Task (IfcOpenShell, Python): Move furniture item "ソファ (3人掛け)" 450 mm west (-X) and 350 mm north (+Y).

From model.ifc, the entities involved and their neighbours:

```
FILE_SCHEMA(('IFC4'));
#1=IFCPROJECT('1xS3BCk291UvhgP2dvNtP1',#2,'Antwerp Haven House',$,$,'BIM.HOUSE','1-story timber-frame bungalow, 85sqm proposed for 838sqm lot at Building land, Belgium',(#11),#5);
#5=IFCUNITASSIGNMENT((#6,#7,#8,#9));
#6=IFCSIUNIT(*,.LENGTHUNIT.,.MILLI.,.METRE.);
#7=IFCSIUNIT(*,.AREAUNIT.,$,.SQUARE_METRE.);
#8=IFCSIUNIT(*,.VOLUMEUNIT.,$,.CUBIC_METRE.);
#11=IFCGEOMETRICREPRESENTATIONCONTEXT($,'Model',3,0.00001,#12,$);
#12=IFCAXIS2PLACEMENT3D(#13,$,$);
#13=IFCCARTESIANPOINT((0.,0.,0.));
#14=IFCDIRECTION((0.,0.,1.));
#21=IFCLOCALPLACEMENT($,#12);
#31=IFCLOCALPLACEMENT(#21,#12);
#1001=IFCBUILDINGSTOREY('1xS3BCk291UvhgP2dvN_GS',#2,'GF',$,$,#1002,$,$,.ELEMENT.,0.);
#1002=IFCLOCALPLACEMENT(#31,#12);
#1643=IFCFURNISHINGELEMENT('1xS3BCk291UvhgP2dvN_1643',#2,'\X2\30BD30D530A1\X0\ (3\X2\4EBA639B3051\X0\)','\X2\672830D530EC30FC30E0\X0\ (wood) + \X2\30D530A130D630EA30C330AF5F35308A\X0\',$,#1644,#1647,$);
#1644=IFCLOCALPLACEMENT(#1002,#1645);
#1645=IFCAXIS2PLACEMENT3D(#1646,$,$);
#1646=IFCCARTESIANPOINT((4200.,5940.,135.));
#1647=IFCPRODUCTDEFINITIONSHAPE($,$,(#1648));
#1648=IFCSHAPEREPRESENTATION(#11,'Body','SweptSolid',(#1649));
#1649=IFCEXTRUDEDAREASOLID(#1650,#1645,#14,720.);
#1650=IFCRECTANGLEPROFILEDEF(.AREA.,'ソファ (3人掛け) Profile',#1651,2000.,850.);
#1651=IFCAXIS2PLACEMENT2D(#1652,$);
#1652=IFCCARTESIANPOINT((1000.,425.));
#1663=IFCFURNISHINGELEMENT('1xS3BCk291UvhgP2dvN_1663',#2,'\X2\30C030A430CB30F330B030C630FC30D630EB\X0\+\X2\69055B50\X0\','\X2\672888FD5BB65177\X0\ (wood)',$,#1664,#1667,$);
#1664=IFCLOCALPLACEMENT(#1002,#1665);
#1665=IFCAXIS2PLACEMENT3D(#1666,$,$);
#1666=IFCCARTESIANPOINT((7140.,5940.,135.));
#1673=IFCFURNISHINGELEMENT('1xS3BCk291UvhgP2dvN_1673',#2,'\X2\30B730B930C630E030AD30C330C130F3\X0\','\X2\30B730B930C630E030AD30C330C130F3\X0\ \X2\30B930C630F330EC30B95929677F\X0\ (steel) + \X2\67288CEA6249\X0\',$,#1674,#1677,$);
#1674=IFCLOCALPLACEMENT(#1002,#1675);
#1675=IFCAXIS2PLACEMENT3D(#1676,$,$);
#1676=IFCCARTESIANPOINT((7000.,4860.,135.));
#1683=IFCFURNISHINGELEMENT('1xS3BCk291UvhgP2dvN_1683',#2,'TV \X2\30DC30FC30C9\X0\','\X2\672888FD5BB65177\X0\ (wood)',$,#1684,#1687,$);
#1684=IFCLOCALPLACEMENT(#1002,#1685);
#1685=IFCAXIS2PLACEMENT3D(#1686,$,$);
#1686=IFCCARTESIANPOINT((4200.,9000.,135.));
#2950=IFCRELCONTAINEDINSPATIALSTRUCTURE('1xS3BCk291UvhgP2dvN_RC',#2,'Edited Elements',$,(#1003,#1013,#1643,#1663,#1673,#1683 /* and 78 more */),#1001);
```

```python
import ifcopenshell
import ifcopenshell.api.geometry
import ifcopenshell.util.placement
import ifcopenshell.util.unit

model = ifcopenshell.open("model.ifc")
unit_scale = ifcopenshell.util.unit.calculate_unit_scale(model)

item = model.by_guid("1xS3BCk291UvhgP2dvN_1643")
matrix = ifcopenshell.util.placement.get_local_placement(item.ObjectPlacement)
matrix[0, 3] -= 0.45 / unit_scale
matrix[1, 3] += 0.35 / unit_scale
ifcopenshell.api.geometry.edit_object_placement(model, product=item, matrix=matrix, is_si=False)

print(ifcopenshell.util.placement.get_local_placement(item.ObjectPlacement).round(3) + 0.0)

model.write("model-out.ifc")
```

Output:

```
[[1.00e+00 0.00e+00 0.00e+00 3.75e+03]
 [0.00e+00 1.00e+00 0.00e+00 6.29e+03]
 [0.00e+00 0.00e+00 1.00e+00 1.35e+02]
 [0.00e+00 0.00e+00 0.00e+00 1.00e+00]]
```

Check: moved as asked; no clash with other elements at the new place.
